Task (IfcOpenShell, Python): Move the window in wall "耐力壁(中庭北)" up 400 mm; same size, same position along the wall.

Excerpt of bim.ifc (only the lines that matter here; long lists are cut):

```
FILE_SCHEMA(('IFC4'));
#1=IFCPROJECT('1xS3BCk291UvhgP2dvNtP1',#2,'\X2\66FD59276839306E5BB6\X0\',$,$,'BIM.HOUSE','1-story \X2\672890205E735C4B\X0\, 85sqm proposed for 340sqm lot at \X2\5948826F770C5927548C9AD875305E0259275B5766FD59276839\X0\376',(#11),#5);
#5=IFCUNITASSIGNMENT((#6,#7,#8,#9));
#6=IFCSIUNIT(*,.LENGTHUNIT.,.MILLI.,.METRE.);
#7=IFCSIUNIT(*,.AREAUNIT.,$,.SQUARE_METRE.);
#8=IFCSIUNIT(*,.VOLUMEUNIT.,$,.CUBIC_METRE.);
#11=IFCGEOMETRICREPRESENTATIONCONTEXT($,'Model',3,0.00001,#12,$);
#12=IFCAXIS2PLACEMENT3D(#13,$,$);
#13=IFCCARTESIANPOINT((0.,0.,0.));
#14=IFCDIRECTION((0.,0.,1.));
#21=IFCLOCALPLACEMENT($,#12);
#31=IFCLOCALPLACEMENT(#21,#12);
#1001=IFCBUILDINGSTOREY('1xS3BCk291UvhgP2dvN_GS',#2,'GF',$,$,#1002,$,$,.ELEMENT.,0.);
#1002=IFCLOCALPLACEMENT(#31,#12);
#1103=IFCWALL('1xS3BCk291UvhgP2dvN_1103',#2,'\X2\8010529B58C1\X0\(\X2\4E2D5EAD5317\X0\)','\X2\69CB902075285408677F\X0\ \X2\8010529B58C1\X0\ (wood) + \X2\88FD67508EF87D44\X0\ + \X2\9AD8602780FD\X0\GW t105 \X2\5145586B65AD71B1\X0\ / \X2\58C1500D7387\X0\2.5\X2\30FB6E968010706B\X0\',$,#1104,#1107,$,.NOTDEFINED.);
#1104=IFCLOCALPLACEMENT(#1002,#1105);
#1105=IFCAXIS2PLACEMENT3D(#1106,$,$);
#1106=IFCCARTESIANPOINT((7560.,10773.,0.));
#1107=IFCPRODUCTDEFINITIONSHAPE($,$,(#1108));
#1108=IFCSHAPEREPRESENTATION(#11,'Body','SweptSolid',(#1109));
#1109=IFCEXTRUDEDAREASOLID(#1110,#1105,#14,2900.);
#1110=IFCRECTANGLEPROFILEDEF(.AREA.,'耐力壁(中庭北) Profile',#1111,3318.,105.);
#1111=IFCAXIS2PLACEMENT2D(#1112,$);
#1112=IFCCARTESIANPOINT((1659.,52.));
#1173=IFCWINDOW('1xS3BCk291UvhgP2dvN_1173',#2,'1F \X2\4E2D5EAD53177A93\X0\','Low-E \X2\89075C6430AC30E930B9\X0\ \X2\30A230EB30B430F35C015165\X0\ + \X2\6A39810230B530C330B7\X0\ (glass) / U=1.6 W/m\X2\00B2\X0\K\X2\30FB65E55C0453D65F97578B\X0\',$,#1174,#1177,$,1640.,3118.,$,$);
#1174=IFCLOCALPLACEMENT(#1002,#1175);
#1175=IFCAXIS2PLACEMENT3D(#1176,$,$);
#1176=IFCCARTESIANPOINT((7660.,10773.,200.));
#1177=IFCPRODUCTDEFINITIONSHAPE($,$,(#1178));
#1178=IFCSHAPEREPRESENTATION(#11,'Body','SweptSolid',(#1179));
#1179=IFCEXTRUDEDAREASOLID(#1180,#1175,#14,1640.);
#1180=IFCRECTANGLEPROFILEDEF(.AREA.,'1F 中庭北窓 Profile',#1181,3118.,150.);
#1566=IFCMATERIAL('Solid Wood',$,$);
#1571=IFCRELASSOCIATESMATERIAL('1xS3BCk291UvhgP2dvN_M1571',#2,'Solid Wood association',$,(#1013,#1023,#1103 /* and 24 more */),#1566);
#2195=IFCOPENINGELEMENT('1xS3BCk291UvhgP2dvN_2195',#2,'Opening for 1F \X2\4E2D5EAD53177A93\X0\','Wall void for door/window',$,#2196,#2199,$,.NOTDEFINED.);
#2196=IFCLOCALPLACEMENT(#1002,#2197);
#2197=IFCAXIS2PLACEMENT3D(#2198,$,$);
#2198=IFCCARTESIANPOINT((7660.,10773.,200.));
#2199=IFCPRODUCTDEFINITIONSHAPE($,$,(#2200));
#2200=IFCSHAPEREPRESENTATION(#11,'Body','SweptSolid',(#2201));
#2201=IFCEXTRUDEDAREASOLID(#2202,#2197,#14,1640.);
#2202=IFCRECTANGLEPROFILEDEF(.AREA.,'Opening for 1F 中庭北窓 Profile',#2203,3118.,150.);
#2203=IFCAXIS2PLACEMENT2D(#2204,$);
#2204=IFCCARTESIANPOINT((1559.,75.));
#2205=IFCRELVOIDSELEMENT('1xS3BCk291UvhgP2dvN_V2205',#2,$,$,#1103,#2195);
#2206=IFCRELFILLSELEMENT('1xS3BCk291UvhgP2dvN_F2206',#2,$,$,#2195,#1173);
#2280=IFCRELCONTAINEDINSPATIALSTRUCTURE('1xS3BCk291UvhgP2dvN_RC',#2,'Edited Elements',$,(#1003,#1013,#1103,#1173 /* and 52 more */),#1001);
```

```python
import numpy as np
import ifcopenshell
import ifcopenshell.api.geometry
import ifcopenshell.util.placement
import ifcopenshell.util.unit

model = ifcopenshell.open("bim.ifc")
unit_scale = ifcopenshell.util.unit.calculate_unit_scale(model)

window = model.by_guid("1xS3BCk291UvhgP2dvN_1173")
opening = window.FillsVoids[0].RelatingOpeningElement
dz = 0.4 / unit_scale

shift = np.array([0.0, 0.0, dz])
# The window is not placed relative to its opening, so move both.
for product in (opening, window):
    matrix = ifcopenshell.util.placement.get_local_placement(product.ObjectPlacement)
    matrix[:3, 3] += shift
    ifcopenshell.api.geometry.edit_object_placement(model, product=product, matrix=matrix, is_si=False)

print(f"moved by {dz * unit_scale:+.3f} m")

model.write("bim_updated.ifc")
```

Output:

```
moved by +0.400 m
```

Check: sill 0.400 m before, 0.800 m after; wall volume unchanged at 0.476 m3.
